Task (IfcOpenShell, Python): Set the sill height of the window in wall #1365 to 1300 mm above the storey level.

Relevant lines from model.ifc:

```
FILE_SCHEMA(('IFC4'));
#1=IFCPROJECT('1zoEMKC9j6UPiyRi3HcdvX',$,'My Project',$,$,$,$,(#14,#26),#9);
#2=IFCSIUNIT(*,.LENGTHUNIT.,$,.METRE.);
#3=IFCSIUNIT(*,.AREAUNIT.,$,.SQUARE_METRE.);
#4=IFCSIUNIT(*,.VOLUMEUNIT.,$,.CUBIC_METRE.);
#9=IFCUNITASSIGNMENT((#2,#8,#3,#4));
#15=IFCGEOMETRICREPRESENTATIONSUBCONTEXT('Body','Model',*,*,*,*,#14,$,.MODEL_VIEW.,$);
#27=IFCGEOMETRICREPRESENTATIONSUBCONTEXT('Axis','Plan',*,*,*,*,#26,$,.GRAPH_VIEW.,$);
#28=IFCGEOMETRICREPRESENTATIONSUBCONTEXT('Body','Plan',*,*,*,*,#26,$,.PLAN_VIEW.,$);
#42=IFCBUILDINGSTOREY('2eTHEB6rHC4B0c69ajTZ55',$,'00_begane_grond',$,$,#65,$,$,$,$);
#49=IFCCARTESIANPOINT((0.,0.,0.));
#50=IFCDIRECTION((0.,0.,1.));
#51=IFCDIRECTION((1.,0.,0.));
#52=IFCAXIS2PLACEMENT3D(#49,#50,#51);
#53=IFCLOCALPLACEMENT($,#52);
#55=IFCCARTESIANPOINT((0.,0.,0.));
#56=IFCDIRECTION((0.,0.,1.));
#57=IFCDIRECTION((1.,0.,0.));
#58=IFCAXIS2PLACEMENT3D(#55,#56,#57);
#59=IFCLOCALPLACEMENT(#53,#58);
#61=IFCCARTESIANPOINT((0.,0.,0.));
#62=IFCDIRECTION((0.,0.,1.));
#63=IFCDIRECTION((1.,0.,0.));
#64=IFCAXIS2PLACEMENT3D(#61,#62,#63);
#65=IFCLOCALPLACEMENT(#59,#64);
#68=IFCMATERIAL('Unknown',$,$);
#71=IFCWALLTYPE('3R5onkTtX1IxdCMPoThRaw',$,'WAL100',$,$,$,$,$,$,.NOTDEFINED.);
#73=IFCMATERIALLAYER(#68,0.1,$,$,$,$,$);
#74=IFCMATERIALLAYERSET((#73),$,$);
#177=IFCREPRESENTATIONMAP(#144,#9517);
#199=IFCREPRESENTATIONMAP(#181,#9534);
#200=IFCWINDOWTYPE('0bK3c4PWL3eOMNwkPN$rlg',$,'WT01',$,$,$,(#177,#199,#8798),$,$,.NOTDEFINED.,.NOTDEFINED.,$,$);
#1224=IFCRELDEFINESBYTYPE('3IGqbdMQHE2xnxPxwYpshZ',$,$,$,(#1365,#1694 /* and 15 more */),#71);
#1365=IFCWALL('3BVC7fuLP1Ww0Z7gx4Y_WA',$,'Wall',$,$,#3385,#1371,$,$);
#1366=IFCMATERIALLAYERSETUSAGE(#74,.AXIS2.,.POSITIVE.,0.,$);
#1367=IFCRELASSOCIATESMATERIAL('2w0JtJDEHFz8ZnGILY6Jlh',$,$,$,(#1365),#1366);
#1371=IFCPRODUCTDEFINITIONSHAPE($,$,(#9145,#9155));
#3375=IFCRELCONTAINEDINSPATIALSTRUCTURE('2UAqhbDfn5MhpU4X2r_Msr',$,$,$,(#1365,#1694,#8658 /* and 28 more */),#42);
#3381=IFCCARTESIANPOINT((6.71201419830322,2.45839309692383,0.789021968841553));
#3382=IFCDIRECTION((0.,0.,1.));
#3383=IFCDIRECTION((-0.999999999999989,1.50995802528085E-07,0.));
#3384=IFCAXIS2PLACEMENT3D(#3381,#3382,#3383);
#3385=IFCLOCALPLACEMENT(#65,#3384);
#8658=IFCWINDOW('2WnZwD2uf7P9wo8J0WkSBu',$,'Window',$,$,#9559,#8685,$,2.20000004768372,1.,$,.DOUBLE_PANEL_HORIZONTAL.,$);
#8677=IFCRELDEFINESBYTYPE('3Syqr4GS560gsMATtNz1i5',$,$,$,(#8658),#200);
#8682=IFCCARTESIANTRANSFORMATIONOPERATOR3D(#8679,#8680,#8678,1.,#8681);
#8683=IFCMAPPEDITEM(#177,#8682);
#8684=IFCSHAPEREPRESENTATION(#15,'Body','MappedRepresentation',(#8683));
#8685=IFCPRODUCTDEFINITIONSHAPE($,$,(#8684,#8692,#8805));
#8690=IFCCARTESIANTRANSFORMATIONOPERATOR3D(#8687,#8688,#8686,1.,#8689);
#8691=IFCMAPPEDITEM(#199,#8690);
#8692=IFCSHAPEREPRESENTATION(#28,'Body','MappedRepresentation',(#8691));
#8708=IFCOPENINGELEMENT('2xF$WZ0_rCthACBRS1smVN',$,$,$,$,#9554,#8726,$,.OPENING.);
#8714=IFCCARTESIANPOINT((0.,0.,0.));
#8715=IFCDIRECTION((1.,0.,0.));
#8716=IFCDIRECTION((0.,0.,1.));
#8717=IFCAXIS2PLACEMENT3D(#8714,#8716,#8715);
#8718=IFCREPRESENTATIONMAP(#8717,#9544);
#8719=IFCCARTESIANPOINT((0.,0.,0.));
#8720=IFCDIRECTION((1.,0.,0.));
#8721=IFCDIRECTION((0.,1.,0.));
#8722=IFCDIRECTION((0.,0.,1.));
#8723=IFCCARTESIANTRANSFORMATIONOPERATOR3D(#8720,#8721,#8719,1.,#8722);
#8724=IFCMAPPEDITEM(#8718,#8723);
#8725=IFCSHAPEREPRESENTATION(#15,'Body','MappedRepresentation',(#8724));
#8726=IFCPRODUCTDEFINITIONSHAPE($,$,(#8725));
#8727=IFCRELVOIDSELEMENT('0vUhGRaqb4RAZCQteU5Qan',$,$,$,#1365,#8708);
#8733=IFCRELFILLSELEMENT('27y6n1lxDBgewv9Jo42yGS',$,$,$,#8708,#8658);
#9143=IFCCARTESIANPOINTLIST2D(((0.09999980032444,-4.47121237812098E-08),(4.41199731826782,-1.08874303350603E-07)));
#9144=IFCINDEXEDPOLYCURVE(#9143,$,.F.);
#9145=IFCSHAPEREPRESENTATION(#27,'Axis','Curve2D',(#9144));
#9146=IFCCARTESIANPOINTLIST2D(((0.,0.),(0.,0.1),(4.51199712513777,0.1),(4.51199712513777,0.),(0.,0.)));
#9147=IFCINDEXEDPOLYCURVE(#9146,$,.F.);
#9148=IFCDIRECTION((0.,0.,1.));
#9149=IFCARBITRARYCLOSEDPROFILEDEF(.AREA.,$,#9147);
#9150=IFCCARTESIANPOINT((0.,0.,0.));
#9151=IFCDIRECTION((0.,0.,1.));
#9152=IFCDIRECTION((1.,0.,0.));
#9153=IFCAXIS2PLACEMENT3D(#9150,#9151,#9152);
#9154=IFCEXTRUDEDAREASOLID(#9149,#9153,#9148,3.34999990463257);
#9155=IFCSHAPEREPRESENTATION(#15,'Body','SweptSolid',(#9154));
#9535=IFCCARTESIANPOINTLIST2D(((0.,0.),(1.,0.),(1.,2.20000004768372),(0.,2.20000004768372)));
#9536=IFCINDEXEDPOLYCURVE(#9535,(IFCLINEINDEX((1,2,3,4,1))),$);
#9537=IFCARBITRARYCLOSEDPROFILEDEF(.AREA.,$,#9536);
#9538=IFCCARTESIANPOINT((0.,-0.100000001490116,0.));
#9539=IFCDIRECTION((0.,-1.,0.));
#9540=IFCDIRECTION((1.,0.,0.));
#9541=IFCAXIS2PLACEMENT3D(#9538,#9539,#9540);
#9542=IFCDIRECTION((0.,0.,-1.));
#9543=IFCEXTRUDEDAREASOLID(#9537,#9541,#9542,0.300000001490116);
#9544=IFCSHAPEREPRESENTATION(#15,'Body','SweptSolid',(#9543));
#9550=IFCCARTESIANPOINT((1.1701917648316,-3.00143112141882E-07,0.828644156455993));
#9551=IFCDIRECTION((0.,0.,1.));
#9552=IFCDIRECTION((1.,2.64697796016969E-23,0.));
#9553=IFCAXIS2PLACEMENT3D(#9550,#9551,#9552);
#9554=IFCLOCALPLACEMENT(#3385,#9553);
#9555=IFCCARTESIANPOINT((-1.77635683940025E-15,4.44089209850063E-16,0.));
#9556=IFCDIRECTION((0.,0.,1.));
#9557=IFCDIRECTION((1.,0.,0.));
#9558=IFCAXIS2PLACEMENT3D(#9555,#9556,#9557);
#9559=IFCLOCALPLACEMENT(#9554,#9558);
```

```python
import numpy as np
import ifcopenshell
import ifcopenshell.api.geometry
import ifcopenshell.geom
import ifcopenshell.util.element
import ifcopenshell.util.placement
import ifcopenshell.util.shape
import ifcopenshell.util.unit

model = ifcopenshell.open("model.ifc")
unit_scale = ifcopenshell.util.unit.calculate_unit_scale(model)

window = model.by_guid("2WnZwD2uf7P9wo8J0WkSBu")
opening = window.FillsVoids[0].RelatingOpeningElement
storey = ifcopenshell.util.element.get_container(window, ifc_class="IfcBuildingStorey")
level = ifcopenshell.util.placement.get_local_placement(storey.ObjectPlacement)[2, 3]

# The opening's origin need not be at the sill, so measure its lowest point.
shape = ifcopenshell.geom.create_shape(ifcopenshell.geom.settings(), opening)
bottom = ifcopenshell.util.shape.get_shape_bottom_elevation(shape, shape.geometry) / unit_scale
dz = level + 1.3 / unit_scale - bottom

shift = np.array([0.0, 0.0, dz])
# The window is placed relative to its opening, so it follows when the opening moves.
matrix = ifcopenshell.util.placement.get_local_placement(opening.ObjectPlacement)
matrix[:3, 3] += shift
ifcopenshell.api.geometry.edit_object_placement(
    model, product=opening, matrix=matrix, is_si=False, should_transform_children=True
)

print(f"moved by {dz * unit_scale:+.3f} m")

model.write("model_edited.ifc")
```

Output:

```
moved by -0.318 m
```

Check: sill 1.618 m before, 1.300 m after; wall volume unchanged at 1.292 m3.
